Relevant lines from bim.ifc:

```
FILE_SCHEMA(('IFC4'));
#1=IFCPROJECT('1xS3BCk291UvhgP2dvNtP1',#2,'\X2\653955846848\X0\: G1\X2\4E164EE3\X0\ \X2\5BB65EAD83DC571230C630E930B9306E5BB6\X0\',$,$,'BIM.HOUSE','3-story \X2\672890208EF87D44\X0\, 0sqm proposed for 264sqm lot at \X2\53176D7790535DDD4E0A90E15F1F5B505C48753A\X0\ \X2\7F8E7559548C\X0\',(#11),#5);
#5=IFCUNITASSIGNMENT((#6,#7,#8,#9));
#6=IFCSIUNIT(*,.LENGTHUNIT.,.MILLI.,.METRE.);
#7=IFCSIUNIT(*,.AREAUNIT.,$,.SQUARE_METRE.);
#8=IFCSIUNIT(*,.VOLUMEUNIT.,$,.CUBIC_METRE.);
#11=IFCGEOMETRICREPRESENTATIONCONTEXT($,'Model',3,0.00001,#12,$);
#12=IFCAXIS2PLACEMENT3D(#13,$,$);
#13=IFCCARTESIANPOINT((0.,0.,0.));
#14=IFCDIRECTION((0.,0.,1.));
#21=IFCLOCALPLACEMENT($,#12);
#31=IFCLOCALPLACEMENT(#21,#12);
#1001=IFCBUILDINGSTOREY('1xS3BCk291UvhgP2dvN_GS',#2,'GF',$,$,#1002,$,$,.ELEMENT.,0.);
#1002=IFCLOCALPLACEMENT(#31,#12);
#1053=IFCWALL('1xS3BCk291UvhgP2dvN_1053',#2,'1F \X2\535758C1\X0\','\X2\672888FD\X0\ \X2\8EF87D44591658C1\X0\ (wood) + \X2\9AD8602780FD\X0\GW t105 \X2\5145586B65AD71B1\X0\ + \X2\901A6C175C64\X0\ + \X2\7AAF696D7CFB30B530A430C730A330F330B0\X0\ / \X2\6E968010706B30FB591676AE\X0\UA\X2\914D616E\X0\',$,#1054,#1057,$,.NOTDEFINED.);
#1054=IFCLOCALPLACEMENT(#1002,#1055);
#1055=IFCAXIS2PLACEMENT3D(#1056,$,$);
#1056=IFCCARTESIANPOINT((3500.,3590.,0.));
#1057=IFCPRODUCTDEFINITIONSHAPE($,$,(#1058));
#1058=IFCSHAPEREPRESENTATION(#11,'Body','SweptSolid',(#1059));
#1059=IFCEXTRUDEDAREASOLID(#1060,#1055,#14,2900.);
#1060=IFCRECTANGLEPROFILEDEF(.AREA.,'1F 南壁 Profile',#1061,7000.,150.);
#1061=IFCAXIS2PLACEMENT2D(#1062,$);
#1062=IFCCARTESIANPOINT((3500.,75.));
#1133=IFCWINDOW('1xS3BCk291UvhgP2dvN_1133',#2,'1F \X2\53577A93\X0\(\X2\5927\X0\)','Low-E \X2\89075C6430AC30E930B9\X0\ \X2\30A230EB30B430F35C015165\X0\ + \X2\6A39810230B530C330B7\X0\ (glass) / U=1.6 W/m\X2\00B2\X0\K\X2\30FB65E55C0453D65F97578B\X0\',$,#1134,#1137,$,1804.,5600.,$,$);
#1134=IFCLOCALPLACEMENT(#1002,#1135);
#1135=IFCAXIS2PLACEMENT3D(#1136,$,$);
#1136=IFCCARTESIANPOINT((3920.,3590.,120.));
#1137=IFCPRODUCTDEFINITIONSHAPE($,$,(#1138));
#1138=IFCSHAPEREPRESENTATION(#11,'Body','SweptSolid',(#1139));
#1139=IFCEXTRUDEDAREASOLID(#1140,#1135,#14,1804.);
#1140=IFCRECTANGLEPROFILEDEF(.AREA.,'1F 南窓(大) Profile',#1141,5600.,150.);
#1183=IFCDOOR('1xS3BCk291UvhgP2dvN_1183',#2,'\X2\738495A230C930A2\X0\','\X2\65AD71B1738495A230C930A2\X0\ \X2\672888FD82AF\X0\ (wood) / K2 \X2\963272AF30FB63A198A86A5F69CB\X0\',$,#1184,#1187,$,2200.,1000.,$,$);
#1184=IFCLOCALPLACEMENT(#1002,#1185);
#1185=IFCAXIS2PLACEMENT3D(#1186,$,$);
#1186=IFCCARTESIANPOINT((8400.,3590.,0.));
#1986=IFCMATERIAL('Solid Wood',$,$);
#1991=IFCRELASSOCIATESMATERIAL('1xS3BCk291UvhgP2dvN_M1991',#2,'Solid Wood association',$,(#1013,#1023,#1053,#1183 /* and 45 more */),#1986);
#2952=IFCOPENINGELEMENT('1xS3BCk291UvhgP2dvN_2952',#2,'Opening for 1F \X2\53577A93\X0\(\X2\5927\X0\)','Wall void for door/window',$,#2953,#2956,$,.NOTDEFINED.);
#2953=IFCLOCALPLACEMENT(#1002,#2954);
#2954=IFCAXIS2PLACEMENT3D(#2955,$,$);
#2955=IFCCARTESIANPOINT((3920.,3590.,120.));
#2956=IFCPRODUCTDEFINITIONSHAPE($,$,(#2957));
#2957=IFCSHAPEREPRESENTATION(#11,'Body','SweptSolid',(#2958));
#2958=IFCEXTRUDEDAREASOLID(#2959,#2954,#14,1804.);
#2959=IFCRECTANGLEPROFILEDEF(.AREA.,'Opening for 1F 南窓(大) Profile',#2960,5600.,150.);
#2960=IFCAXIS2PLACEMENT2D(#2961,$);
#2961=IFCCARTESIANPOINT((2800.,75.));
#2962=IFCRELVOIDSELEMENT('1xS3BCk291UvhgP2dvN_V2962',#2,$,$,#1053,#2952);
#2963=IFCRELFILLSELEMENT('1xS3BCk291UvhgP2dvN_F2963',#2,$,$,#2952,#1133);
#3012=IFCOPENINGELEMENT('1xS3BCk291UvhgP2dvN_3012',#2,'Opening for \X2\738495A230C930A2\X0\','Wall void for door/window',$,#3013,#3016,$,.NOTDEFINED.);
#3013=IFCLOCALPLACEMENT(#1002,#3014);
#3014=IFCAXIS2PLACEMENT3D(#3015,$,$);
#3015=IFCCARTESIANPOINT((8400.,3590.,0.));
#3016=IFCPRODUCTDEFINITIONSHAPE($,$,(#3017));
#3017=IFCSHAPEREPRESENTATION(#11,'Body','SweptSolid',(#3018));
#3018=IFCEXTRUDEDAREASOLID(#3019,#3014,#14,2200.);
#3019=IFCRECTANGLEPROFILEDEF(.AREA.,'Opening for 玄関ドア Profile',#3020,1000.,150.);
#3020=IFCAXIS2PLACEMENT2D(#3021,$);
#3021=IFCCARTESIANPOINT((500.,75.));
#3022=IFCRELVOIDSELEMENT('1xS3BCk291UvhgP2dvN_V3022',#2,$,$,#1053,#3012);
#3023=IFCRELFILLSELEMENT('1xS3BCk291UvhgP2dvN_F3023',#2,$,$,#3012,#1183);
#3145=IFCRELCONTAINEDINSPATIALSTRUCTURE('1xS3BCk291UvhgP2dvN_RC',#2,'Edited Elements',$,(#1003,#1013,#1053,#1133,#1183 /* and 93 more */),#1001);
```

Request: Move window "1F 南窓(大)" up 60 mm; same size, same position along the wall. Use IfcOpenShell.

```python
import numpy as np
import ifcopenshell
import ifcopenshell.api.geometry
import ifcopenshell.util.placement
import ifcopenshell.util.unit

model = ifcopenshell.open("bim.ifc")
unit_scale = ifcopenshell.util.unit.calculate_unit_scale(model)

window = model.by_id(1133)
opening = window.FillsVoids[0].RelatingOpeningElement
dz = 0.06 / unit_scale

shift = np.array([0.0, 0.0, dz])
# The window is not placed relative to its opening, so move both.
for product in (opening, window):
    matrix = ifcopenshell.util.placement.get_local_placement(product.ObjectPlacement)
    matrix[:3, 3] += shift
    ifcopenshell.api.geometry.edit_object_placement(model, product=product, matrix=matrix, is_si=False)

print(f"moved by {dz * unit_scale:+.3f} m")

model.write("bim_v2.ifc")
```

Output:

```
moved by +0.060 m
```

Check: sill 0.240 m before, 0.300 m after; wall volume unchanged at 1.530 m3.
